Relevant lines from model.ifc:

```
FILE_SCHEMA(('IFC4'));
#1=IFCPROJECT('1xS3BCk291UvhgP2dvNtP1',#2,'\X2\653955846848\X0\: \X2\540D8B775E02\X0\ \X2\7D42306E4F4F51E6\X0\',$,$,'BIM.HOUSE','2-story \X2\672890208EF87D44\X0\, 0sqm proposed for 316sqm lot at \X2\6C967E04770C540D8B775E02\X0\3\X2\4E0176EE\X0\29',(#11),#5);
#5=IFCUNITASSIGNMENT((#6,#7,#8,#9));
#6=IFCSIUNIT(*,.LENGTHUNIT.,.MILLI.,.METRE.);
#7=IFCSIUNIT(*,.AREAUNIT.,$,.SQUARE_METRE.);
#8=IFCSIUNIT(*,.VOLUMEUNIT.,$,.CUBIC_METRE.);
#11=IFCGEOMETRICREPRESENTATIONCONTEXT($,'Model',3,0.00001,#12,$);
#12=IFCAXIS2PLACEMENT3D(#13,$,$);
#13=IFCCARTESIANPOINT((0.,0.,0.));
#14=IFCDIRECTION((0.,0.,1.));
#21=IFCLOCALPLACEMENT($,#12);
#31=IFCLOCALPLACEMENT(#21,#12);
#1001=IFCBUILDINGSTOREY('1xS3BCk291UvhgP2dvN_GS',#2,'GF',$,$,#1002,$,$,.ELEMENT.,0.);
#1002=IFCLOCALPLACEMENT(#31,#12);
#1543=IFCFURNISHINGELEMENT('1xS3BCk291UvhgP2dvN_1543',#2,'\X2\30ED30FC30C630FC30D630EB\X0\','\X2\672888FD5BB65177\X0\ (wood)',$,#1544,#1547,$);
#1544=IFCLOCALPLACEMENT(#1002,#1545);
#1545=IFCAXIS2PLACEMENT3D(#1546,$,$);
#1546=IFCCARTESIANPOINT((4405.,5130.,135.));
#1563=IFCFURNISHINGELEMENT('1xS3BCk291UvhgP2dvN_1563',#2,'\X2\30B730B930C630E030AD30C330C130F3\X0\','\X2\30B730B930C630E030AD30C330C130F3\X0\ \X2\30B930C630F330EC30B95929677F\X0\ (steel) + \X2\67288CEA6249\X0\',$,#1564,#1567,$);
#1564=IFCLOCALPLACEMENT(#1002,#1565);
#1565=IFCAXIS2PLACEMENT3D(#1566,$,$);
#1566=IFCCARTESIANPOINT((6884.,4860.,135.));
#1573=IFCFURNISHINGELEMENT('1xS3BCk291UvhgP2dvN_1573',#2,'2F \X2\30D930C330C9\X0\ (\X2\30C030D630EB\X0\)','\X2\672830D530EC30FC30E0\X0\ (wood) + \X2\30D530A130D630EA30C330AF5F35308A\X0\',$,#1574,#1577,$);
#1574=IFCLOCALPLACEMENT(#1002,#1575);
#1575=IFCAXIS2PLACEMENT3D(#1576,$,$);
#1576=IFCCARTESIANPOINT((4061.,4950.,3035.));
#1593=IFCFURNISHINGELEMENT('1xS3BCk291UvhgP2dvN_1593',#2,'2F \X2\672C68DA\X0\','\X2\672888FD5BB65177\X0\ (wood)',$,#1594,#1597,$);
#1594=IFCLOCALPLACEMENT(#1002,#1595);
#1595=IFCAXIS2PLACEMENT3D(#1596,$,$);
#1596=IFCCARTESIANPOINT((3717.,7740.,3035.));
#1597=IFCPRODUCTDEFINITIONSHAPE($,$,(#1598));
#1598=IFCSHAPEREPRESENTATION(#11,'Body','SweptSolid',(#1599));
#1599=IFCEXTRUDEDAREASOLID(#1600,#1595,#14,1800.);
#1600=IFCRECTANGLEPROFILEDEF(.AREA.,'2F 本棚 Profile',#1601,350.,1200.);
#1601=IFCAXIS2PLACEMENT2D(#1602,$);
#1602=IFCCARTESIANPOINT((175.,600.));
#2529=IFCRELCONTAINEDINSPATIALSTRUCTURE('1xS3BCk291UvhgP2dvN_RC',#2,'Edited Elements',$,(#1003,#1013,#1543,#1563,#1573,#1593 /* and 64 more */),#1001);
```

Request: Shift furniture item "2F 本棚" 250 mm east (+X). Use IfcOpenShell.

```python
import ifcopenshell
import ifcopenshell.api.geometry
import ifcopenshell.util.placement
import ifcopenshell.util.unit

model = ifcopenshell.open("model.ifc")
unit_scale = ifcopenshell.util.unit.calculate_unit_scale(model)

item = model.by_guid("1xS3BCk291UvhgP2dvN_1593")
matrix = ifcopenshell.util.placement.get_local_placement(item.ObjectPlacement)
matrix[0, 3] += 0.25 / unit_scale
ifcopenshell.api.geometry.edit_object_placement(model, product=item, matrix=matrix, is_si=False)

print(ifcopenshell.util.placement.get_local_placement(item.ObjectPlacement).round(3) + 0.0)

model.write("model_updated.ifc")
```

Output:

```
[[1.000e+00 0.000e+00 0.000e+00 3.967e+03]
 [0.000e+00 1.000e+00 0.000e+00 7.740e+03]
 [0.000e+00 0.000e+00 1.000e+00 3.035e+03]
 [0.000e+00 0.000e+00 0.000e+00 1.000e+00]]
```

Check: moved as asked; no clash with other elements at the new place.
